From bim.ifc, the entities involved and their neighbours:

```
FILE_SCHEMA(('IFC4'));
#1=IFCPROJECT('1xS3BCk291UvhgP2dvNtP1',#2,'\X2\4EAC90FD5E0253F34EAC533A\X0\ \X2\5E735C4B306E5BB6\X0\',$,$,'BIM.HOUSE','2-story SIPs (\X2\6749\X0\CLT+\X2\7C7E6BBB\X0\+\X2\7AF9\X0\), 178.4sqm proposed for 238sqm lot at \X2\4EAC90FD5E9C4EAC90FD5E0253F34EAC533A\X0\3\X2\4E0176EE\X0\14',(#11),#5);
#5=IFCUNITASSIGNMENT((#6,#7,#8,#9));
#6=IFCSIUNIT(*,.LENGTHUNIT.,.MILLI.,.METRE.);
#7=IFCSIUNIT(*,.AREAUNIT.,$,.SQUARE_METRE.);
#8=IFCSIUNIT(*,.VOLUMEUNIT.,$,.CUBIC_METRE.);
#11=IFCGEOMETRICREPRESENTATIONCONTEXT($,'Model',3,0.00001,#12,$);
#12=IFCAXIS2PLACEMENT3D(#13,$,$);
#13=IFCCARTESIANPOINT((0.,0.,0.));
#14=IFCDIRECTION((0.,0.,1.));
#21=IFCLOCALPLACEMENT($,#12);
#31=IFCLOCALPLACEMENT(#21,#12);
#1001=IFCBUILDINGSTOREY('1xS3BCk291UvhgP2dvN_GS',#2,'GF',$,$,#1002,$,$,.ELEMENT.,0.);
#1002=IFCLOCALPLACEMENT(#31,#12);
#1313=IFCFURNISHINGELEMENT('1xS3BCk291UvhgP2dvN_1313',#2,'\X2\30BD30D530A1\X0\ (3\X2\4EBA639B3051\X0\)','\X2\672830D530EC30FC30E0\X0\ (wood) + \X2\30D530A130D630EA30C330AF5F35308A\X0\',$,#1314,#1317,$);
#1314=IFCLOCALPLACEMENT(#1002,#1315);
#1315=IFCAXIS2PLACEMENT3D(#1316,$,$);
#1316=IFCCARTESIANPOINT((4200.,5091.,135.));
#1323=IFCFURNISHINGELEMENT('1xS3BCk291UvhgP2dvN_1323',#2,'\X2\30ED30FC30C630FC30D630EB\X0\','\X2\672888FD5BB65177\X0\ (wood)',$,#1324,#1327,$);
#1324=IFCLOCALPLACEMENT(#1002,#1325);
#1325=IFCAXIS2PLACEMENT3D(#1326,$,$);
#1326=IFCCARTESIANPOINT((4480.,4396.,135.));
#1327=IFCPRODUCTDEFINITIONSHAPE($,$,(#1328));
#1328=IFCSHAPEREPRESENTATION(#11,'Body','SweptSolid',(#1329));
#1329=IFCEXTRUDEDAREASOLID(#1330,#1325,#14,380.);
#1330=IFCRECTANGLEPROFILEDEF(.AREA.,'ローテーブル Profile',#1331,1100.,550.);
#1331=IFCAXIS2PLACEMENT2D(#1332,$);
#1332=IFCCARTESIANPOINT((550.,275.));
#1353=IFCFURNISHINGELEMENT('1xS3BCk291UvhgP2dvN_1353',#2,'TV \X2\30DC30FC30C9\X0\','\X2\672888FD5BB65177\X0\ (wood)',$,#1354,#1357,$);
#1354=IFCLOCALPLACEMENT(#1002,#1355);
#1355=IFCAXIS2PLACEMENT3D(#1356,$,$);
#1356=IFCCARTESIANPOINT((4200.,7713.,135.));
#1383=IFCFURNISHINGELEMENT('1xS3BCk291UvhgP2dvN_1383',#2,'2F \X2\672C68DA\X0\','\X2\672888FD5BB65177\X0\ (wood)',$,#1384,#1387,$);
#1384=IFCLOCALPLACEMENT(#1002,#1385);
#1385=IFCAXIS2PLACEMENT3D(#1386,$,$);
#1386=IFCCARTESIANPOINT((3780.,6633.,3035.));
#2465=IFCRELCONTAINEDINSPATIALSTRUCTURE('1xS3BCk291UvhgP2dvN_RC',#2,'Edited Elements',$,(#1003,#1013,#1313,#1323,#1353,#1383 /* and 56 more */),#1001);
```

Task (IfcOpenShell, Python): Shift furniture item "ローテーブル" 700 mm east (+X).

```python
import ifcopenshell
import ifcopenshell.api.geometry
import ifcopenshell.util.placement

model = ifcopenshell.open("bim.ifc")

item = model.by_guid("1xS3BCk291UvhgP2dvN_1323")
matrix = ifcopenshell.util.placement.get_local_placement(item.ObjectPlacement)
matrix[0, 3] += 700.0
ifcopenshell.api.geometry.edit_object_placement(model, product=item, matrix=matrix, is_si=False)

print(ifcopenshell.util.placement.get_local_placement(item.ObjectPlacement).round(3) + 0.0)

model.write("bim_v2.ifc")
```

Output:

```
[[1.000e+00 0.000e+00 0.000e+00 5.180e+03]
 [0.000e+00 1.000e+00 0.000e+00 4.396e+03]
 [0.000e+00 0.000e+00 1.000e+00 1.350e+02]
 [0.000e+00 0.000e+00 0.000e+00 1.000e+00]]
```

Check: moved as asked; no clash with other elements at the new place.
